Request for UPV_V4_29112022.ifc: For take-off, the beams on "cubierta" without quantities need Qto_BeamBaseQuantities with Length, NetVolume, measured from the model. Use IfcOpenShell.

First a look at what the model holds.

```python
import ifcopenshell
import ifcopenshell.util.element
import ifcopenshell.util.unit

model = ifcopenshell.open("UPV_V4_29112022.ifc")
print(model.schema)
for unit_type in ("LENGTHUNIT", "AREAUNIT", "VOLUMEUNIT"):
    print(unit_type, ifcopenshell.util.unit.calculate_unit_scale(model, unit_type))
storey = next(s for s in model.by_type("IfcBuildingStorey") if s.Name == "cubierta")
beams = [e for e in ifcopenshell.util.element.get_decomposition(storey) if e.is_a("IfcBeam")]
for e in sorted(beams, key=lambda e: e.id()):
    print(e.id(), e.is_a(), e.Name, list(ifcopenshell.util.element.get_psets(e, qtos_only=True)), sep=" | ")
```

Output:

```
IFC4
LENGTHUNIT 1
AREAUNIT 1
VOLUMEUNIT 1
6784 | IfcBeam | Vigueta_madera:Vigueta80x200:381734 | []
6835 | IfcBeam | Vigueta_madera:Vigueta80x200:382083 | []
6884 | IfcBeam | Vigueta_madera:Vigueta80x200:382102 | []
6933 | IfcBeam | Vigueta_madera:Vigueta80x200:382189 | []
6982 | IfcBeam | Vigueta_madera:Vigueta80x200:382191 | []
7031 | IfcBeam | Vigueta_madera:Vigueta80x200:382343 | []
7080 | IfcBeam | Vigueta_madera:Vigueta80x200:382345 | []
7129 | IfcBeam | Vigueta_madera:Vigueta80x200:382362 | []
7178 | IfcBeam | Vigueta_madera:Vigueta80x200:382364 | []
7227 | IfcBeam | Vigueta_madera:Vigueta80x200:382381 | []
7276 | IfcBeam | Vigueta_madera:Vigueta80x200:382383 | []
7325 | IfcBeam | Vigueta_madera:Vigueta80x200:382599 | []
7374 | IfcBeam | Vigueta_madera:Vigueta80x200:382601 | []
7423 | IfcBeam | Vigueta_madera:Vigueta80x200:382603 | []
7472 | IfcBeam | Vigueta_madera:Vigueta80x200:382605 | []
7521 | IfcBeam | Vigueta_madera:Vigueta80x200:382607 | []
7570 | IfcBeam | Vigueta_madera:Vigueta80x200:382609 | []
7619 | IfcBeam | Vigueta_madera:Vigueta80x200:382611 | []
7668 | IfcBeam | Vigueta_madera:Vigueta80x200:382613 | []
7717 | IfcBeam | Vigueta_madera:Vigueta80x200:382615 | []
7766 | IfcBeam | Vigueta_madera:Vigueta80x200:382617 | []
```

```python
import ifcopenshell
import ifcopenshell.api.pset
import ifcopenshell.geom
import ifcopenshell.util.element
import ifcopenshell.util.shape
import ifcopenshell.util.unit

model = ifcopenshell.open("UPV_V4_29112022.ifc")
unit_scale = ifcopenshell.util.unit.calculate_unit_scale(model)
volume_scale = ifcopenshell.util.unit.calculate_unit_scale(model, "VOLUMEUNIT")
settings = ifcopenshell.geom.settings()

storey = next(s for s in model.by_type("IfcBuildingStorey") if s.Name == "cubierta")
beams = [e for e in ifcopenshell.util.element.get_decomposition(storey) if e.is_a("IfcBeam")]

for e in sorted(beams, key=lambda e: e.id()):
    if ifcopenshell.util.element.get_psets(e, qtos_only=True, should_inherit=False):
        continue
    # Geometry comes back in metres, in the element's own axes.
    shape = ifcopenshell.geom.create_shape(settings, e)
    values = {
        "Length": ifcopenshell.util.shape.get_max_xyz(shape.geometry) / unit_scale,
        "NetVolume": ifcopenshell.util.shape.get_volume(shape.geometry) / volume_scale,
    }
    qto = ifcopenshell.api.pset.add_qto(model, product=e, name="Qto_BeamBaseQuantities")
    ifcopenshell.api.pset.edit_qto(model, qto=qto, properties=values)
    print(e.id(), {k: round(v, 3) for k, v in values.items()})

model.write("UPV_V4_29112022_edited.ifc")
```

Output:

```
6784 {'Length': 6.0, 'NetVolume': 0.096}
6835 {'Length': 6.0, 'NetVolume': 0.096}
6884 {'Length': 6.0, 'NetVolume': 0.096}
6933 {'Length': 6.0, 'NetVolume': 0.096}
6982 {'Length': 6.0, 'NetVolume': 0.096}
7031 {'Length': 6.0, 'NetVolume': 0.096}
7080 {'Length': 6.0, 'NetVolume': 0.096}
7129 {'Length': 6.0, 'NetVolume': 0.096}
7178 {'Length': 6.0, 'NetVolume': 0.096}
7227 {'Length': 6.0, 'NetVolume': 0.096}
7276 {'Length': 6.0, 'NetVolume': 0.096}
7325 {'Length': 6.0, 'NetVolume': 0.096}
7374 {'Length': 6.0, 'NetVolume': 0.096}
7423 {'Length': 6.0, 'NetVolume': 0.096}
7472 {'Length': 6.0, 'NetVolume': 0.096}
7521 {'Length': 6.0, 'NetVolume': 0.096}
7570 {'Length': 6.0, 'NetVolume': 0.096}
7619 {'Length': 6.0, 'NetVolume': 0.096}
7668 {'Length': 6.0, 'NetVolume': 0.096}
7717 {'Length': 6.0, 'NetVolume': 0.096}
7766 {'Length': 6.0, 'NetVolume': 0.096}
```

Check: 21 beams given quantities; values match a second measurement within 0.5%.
